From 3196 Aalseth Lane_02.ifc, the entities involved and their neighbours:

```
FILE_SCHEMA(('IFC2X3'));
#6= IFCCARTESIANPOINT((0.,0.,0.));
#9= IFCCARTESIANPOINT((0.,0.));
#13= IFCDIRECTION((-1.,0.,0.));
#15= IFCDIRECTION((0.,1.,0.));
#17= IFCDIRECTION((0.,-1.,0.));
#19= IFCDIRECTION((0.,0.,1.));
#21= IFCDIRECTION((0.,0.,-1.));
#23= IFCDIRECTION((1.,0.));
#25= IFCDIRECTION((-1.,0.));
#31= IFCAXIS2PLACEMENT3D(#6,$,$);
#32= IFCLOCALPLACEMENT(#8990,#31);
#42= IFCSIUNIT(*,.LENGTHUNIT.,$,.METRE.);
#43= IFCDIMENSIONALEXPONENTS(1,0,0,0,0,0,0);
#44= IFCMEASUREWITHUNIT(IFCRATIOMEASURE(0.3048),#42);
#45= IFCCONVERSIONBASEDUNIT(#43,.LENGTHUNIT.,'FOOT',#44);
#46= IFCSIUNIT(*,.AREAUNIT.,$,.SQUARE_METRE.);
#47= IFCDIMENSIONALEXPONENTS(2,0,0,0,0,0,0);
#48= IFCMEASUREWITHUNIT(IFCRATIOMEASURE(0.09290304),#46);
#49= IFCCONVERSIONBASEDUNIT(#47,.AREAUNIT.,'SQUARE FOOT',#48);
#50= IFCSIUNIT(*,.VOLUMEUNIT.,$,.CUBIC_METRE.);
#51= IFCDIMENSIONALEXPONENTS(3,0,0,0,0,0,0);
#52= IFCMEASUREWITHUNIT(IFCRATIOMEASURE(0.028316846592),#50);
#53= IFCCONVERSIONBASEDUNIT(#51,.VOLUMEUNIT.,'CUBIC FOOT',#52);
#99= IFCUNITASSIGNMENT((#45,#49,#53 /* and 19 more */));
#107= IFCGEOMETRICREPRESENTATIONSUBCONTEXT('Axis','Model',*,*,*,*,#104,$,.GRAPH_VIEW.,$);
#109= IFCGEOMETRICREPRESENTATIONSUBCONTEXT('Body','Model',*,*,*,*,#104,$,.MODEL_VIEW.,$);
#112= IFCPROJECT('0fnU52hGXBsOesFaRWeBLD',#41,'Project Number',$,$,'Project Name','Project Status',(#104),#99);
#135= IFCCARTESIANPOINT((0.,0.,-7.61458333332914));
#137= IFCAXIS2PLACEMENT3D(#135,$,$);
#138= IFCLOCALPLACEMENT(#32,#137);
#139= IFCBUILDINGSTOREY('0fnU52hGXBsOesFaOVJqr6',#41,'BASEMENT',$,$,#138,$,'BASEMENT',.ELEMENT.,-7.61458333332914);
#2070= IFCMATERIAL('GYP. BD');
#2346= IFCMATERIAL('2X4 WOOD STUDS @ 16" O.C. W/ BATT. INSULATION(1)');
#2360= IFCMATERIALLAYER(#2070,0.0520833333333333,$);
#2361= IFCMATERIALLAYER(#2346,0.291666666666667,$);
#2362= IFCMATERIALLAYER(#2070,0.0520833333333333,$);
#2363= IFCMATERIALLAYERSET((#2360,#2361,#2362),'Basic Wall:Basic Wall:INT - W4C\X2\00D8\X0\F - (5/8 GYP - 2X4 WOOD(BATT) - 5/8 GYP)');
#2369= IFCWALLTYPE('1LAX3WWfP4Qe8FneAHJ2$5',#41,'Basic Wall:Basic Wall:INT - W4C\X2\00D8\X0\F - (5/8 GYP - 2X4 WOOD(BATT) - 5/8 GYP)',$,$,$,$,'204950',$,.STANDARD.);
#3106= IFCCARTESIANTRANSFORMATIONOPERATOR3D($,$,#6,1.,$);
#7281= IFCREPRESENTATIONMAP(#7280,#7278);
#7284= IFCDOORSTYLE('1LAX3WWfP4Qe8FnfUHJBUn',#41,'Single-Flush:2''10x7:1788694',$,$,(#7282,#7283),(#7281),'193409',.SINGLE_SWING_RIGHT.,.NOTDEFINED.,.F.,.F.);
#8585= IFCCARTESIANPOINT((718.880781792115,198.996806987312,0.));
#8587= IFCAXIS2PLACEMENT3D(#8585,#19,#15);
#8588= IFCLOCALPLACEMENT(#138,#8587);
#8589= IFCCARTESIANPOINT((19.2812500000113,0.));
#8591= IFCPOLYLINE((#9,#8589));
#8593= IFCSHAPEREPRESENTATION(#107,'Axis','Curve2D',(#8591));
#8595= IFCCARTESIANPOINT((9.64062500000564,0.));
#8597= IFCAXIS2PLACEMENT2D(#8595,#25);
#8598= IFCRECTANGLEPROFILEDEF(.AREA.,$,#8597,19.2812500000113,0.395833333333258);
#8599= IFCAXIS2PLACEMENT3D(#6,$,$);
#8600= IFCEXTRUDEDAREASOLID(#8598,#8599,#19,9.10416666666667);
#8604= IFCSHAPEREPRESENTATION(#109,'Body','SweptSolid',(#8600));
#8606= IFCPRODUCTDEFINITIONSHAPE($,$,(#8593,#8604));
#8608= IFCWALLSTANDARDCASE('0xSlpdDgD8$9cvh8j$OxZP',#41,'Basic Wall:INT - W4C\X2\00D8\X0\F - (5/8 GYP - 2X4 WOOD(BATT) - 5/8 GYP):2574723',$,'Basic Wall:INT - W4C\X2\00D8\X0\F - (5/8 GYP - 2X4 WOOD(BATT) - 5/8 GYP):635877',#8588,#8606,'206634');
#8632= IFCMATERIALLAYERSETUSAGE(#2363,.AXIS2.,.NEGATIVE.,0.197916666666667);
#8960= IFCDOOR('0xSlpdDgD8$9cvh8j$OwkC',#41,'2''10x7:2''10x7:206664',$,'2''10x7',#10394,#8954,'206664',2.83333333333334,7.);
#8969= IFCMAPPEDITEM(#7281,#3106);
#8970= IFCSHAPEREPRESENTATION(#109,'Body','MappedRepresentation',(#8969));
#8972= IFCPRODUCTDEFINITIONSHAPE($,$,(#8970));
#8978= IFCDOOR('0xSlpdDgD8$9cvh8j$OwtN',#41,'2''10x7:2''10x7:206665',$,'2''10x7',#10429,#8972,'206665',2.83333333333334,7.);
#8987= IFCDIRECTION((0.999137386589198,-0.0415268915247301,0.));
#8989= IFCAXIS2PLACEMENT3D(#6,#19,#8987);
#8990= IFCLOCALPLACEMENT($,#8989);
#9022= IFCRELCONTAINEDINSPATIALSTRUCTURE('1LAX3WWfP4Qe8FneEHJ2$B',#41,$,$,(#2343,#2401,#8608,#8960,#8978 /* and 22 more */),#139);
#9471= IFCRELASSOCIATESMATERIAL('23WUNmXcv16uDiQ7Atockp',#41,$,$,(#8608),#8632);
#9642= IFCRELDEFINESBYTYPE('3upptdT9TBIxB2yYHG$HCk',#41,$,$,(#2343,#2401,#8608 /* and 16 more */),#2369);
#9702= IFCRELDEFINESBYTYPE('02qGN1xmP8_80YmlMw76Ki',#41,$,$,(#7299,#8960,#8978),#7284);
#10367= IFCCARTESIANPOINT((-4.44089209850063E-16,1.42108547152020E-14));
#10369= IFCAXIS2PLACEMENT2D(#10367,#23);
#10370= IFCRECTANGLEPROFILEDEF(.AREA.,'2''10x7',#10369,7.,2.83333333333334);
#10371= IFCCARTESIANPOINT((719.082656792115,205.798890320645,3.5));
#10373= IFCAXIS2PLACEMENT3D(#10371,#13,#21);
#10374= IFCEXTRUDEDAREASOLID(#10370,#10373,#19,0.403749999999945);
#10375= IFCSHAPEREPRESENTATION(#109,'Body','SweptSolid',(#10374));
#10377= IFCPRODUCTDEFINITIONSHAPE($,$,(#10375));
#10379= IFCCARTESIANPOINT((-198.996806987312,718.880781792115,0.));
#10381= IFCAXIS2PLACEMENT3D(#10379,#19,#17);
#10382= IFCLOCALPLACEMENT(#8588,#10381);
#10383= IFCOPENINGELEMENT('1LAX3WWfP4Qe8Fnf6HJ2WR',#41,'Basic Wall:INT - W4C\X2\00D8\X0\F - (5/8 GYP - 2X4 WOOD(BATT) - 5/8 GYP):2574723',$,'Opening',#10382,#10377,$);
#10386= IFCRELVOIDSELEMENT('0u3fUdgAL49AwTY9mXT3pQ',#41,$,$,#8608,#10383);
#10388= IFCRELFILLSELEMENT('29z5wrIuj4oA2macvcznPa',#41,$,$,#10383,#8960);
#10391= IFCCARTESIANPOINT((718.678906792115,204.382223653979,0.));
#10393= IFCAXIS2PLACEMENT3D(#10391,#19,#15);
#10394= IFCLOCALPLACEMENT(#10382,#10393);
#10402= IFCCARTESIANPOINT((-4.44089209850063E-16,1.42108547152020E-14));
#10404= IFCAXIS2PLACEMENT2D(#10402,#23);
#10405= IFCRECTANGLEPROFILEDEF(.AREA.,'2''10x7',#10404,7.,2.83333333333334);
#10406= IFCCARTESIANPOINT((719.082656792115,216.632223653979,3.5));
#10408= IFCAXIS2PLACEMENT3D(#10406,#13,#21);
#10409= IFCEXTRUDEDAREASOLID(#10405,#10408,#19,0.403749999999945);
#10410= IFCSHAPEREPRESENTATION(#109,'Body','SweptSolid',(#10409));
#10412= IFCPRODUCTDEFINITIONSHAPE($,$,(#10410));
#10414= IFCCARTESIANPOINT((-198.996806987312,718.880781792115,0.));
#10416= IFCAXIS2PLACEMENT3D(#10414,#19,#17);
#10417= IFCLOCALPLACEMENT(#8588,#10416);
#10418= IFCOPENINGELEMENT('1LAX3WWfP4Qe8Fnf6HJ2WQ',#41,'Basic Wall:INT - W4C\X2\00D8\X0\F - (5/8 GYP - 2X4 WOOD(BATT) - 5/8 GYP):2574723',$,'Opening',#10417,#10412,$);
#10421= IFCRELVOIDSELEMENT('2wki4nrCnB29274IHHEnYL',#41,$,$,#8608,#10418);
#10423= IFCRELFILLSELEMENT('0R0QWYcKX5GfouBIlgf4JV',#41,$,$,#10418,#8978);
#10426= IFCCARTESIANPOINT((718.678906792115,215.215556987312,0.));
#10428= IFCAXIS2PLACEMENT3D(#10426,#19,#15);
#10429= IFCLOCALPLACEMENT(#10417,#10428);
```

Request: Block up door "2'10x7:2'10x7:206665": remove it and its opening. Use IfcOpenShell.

```python
import ifcopenshell
import ifcopenshell.api.feature
import ifcopenshell.api.root
import ifcopenshell.geom
import ifcopenshell.util.shape

model = ifcopenshell.open("3196 Aalseth Lane_02.ifc")
settings = ifcopenshell.geom.settings()


def volume(element):
    """Net volume in cubic metres, openings subtracted."""
    shape = ifcopenshell.geom.create_shape(settings, element)
    return ifcopenshell.util.shape.get_volume(shape.geometry)


door = model.by_id(8978)
opening = door.FillsVoids[0].RelatingOpeningElement
wall = opening.VoidsElements[0].RelatingBuildingElement
before = volume(wall)

ifcopenshell.api.root.remove_product(model, product=door)
ifcopenshell.api.feature.remove_feature(model, feature=opening)

after = volume(wall)

print(f"wall volume {before:.3f} -> {after:.3f} m3")

model.write("3196 Aalseth Lane_02_updated.ifc")
```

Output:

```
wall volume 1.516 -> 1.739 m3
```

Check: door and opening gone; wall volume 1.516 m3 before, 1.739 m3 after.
